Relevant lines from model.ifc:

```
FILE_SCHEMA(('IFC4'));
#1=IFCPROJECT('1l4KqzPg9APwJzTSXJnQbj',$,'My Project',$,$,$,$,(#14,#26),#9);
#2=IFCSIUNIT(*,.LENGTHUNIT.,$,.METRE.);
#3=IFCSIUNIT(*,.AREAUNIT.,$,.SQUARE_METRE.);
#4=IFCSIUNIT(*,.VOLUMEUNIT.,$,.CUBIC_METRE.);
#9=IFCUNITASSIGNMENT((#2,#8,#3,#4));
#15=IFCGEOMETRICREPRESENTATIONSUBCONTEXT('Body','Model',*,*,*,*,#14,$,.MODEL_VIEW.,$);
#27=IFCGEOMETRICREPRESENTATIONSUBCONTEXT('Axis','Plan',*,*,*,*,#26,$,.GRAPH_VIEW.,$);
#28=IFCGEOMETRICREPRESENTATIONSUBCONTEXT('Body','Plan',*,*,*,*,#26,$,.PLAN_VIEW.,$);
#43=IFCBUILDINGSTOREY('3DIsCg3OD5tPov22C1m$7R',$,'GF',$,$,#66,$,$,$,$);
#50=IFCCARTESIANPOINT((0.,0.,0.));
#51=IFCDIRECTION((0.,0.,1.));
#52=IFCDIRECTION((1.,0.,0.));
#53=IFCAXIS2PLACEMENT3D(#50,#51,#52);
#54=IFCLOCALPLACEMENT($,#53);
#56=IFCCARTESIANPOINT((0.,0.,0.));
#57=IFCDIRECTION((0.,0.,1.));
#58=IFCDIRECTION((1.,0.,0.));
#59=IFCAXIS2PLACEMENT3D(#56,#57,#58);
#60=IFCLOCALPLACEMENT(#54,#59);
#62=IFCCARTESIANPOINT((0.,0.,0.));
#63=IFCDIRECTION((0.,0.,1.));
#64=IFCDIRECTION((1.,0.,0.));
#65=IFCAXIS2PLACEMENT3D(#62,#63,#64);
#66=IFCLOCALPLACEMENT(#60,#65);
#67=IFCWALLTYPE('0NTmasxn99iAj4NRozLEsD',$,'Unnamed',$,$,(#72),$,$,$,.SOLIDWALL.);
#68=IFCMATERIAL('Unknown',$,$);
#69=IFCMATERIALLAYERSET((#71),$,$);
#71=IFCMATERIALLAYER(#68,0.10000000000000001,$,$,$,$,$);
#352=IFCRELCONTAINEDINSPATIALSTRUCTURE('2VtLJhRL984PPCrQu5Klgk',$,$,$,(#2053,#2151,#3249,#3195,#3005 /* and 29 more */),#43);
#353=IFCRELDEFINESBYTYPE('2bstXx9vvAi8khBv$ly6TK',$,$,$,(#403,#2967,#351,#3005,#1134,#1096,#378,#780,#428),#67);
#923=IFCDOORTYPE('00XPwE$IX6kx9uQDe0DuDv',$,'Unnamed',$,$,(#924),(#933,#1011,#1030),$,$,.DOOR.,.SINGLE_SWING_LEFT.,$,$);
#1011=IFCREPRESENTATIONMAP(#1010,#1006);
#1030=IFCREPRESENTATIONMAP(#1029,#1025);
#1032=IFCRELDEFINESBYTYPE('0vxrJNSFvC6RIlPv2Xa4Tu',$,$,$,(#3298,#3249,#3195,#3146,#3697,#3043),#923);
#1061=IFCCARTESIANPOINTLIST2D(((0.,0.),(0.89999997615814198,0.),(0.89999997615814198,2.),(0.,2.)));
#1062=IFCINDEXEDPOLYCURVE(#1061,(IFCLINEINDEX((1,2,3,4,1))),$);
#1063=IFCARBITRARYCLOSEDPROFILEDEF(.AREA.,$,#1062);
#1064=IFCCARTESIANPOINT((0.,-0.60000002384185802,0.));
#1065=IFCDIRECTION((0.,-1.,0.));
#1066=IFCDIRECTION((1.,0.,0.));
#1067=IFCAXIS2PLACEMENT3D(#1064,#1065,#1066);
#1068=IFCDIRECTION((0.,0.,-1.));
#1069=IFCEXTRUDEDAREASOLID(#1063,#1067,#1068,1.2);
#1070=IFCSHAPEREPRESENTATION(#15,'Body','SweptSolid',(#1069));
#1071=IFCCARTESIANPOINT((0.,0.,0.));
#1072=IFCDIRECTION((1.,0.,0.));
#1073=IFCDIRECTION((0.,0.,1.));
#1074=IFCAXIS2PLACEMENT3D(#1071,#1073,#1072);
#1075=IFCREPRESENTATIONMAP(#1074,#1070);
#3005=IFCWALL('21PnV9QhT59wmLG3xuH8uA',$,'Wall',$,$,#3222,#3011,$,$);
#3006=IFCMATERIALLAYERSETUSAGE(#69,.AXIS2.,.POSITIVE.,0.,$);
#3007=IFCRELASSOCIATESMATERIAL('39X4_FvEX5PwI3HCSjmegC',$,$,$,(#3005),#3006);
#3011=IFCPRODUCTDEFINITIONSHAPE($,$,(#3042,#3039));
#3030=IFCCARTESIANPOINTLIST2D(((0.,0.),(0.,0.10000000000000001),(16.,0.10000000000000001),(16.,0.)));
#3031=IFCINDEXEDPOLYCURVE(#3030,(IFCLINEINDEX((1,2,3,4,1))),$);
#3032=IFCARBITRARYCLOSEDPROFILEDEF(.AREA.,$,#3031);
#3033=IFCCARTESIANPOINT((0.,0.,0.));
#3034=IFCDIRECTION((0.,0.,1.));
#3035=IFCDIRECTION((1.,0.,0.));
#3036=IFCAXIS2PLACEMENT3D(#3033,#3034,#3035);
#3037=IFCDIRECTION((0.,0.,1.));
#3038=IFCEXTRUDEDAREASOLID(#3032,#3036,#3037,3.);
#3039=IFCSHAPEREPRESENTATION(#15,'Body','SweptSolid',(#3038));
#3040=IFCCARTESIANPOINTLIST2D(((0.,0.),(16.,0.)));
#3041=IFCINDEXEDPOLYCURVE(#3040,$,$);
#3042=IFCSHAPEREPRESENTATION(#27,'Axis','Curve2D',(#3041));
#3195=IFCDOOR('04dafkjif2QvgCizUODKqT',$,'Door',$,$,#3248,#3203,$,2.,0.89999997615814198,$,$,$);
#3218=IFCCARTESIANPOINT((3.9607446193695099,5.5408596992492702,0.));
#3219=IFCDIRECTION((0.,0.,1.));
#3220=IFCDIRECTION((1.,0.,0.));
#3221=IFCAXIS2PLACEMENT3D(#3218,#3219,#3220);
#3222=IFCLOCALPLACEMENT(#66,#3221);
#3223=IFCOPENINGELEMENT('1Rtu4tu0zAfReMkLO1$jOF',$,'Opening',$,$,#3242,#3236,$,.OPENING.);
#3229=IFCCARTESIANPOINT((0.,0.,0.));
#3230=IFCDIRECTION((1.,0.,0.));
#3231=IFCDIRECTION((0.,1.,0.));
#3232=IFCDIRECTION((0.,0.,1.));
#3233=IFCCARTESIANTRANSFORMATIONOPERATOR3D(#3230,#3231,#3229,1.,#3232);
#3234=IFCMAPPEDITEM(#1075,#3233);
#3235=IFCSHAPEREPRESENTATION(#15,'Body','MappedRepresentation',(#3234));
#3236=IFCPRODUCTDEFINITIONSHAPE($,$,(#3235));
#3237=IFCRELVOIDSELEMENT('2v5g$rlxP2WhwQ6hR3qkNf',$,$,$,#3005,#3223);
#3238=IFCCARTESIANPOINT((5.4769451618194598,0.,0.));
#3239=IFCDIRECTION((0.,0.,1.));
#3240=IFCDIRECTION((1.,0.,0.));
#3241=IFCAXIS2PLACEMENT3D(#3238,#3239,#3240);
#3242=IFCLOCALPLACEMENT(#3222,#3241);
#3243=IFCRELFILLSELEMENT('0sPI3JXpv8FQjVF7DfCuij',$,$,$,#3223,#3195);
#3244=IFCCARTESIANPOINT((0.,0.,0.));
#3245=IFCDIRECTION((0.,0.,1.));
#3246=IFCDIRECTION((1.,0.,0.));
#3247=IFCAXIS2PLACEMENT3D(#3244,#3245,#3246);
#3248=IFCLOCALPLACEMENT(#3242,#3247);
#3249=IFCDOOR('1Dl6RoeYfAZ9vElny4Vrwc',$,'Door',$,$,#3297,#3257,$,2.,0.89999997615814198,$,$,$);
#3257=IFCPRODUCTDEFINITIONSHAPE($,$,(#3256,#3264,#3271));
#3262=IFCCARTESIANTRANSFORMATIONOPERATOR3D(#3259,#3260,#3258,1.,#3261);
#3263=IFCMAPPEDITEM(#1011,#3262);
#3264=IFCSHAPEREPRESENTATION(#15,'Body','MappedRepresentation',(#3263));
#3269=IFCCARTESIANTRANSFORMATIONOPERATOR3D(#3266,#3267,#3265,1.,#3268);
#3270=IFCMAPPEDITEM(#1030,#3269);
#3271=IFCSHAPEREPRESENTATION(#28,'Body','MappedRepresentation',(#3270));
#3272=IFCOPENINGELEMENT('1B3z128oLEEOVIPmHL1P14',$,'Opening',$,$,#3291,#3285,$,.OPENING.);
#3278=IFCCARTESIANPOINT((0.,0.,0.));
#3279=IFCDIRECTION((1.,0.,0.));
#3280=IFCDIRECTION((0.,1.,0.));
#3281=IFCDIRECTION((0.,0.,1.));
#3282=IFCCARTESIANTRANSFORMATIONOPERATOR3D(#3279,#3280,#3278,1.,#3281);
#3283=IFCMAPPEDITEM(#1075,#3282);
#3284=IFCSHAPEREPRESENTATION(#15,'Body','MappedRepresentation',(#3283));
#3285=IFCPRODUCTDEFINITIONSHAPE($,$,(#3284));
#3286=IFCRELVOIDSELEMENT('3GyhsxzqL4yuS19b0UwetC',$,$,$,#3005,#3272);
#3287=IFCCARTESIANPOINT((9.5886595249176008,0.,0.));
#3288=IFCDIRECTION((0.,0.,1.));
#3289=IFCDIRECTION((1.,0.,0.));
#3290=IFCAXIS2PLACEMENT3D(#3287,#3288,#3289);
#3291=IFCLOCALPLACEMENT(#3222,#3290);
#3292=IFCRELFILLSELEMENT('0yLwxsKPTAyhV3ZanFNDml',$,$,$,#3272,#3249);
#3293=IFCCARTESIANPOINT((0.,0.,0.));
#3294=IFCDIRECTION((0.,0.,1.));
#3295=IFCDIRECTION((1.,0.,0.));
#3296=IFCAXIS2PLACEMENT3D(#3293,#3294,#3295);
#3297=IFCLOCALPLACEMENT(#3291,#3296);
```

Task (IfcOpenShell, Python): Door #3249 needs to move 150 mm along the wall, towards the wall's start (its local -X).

```python
import ifcopenshell
import ifcopenshell.api.geometry
import ifcopenshell.util.placement

model = ifcopenshell.open("model.ifc")

door = model.by_guid("1Dl6RoeYfAZ9vElny4Vrwc")
opening = door.FillsVoids[0].RelatingOpeningElement
wall = opening.VoidsElements[0].RelatingBuildingElement

wall_matrix = ifcopenshell.util.placement.get_local_placement(wall.ObjectPlacement)
shift = wall_matrix[:3, 0] * -0.15
before = ifcopenshell.util.placement.get_local_placement(door.ObjectPlacement)[:3, 3].copy()

# The door is placed relative to its opening, so it follows when the opening moves.
matrix = ifcopenshell.util.placement.get_local_placement(opening.ObjectPlacement)
matrix[:3, 3] += shift
ifcopenshell.api.geometry.edit_object_placement(
    model, product=opening, matrix=matrix, is_si=False, should_transform_children=True
)

after = ifcopenshell.util.placement.get_local_placement(door.ObjectPlacement)[:3, 3]
print("door moved by", (after - before).round(3) + 0.0)

model.write("model-out.ifc")
```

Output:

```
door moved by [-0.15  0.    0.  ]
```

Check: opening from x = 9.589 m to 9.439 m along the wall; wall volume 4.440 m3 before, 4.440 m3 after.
